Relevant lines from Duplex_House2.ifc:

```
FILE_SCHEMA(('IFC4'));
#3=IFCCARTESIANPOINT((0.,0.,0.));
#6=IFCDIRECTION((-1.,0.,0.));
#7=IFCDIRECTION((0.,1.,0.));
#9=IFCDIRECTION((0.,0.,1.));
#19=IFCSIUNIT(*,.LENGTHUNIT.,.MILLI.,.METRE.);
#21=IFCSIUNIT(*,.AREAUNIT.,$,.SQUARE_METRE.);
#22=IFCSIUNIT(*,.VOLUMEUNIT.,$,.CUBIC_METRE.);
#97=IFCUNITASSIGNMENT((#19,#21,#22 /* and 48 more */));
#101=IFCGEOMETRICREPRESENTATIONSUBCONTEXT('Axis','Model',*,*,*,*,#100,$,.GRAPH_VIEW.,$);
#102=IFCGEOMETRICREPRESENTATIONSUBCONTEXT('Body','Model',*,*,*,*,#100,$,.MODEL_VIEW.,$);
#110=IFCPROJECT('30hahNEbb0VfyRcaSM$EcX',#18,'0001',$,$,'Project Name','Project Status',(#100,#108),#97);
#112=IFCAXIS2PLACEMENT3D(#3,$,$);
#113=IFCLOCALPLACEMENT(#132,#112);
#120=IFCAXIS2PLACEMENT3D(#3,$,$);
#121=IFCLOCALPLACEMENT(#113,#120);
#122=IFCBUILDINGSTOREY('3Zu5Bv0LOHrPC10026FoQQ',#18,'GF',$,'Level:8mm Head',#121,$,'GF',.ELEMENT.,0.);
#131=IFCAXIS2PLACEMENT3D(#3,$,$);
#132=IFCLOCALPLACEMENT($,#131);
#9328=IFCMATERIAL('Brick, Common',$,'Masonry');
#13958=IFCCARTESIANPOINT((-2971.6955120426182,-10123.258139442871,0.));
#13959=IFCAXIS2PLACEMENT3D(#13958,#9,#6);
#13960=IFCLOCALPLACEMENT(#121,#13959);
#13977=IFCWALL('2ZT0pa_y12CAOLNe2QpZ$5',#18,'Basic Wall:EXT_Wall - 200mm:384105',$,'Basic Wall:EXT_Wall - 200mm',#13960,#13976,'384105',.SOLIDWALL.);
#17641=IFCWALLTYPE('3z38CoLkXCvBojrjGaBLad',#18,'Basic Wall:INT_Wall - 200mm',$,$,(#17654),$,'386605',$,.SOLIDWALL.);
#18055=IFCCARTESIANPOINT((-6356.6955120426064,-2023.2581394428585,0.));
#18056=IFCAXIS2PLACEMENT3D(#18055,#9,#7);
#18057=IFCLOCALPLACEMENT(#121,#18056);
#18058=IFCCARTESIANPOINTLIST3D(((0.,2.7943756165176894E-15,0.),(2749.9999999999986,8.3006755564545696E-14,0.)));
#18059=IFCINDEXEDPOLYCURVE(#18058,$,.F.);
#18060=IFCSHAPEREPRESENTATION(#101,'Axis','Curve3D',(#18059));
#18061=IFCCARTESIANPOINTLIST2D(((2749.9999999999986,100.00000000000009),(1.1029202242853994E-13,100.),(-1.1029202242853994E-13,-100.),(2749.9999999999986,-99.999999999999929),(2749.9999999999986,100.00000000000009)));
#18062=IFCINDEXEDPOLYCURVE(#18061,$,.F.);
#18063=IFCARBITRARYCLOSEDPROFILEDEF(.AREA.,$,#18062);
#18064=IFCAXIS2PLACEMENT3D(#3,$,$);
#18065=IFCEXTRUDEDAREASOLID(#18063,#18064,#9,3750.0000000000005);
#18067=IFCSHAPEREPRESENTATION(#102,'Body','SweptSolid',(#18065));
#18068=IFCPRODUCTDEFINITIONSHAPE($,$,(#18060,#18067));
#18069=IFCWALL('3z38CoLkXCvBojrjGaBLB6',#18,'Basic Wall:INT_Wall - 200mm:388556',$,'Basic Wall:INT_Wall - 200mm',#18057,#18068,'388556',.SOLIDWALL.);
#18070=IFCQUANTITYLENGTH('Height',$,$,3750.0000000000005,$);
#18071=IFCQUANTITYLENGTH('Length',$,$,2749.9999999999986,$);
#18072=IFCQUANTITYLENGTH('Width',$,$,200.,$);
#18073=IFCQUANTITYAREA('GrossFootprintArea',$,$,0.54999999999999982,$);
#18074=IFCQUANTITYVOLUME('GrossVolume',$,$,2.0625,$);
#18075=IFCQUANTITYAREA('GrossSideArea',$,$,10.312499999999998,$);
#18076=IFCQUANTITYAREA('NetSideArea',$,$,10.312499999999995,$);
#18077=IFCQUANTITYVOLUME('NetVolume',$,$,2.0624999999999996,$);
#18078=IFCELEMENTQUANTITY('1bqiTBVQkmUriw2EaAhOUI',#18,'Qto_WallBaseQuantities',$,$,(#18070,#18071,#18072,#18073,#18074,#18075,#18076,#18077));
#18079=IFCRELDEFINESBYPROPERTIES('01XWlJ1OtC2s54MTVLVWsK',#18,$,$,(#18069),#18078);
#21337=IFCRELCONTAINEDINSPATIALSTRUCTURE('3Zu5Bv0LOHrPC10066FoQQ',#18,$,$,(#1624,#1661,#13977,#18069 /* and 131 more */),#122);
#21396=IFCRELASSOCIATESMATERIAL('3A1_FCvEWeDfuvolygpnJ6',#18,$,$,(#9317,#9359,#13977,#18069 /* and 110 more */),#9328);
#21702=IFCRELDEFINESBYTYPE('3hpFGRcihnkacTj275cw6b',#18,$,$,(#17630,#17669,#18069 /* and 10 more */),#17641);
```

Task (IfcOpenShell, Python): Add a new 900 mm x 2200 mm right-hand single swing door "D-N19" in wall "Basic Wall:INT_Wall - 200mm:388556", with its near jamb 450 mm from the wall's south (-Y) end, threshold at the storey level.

```python
import numpy as np
import ifcopenshell
import ifcopenshell.api.feature
import ifcopenshell.api.geometry
import ifcopenshell.api.pset
import ifcopenshell.api.root
import ifcopenshell.api.spatial
import ifcopenshell.geom
import ifcopenshell.util.element
import ifcopenshell.util.placement
import ifcopenshell.util.representation
import ifcopenshell.util.shape
import ifcopenshell.util.unit

model = ifcopenshell.open("Duplex_House2.ifc")
unit_scale = ifcopenshell.util.unit.calculate_unit_scale(model)
area_scale = ifcopenshell.util.unit.calculate_unit_scale(model, "AREAUNIT")
volume_scale = ifcopenshell.util.unit.calculate_unit_scale(model, "VOLUMEUNIT")
settings = ifcopenshell.geom.settings()


def volume(element):
    """Net volume in cubic metres, openings subtracted."""
    shape = ifcopenshell.geom.create_shape(settings, element)
    return ifcopenshell.util.shape.get_volume(shape.geometry)


wall = model.by_guid("3z38CoLkXCvBojrjGaBLB6")
storey = ifcopenshell.util.element.get_container(wall, ifc_class="IfcBuildingStorey")
context = ifcopenshell.util.representation.get_context(model, "Model", "Body", "MODEL_VIEW")
before = volume(wall)

width, height, from_end, sill = 0.9, 2.2, 0.45, 0.0  # metres

# The wall runs along its own X axis, and the end named is its -X end.
wall_shape = ifcopenshell.geom.create_shape(settings, wall)
x, y, z = ifcopenshell.util.shape.get_vertices(wall_shape.geometry).T
start = x.min() + from_end
face, thickness = float(y.min()), float(y.max() - y.min())
wall_matrix = ifcopenshell.util.placement.get_local_placement(wall.ObjectPlacement)
level = ifcopenshell.util.placement.get_local_placement(storey.ObjectPlacement)[2, 3]


def in_wall(x, y):
    """Placement at x, y metres in the wall's axes, at sill height."""
    matrix = wall_matrix.copy()
    matrix[:, 3] = wall_matrix @ np.array([x / unit_scale, y / unit_scale, 0.0, 1.0])
    matrix[2, 3] = level + sill / unit_scale
    return matrix


# Opening: a box that overshoots both wall faces by 50 mm.
opening = ifcopenshell.api.root.create_entity(model, ifc_class="IfcOpeningElement", predefined_type="OPENING")
box = ifcopenshell.api.geometry.add_wall_representation(
    model, context=context, length=width, height=height, thickness=thickness + 0.1
)
ifcopenshell.api.geometry.assign_representation(model, product=opening, representation=box)
ifcopenshell.api.geometry.edit_object_placement(model, product=opening, matrix=in_wall(start, face - 0.05), is_si=False)
ifcopenshell.api.feature.add_feature(model, feature=opening, element=wall)

door = ifcopenshell.api.root.create_entity(model, ifc_class="IfcDoor", name="D-N19", predefined_type="DOOR")
door.OverallWidth, door.OverallHeight = width / unit_scale, height / unit_scale
door.OperationType = "SINGLE_SWING_RIGHT"
body = ifcopenshell.api.geometry.add_door_representation(
    model,
    context=context,
    overall_width=door.OverallWidth,
    overall_height=door.OverallHeight,
    operation_type="SINGLE_SWING_RIGHT",
    lining_properties={"LiningDepth": thickness / unit_scale, "ThresholdDepth": thickness / unit_scale},
)
ifcopenshell.api.geometry.assign_representation(model, product=door, representation=body)
ifcopenshell.api.spatial.assign_container(model, products=[door], relating_structure=storey)
ifcopenshell.api.feature.add_filling(model, opening=opening, element=door)

# The lining spans the wall, so the door starts at the wall face.
ifcopenshell.api.geometry.edit_object_placement(model, product=door, matrix=in_wall(start, face), is_si=False)

after = volume(wall)

# Update the wall's stored quantities.
qto = model.by_id(ifcopenshell.util.element.get_pset(wall, "Qto_WallBaseQuantities", should_inherit=False)["id"])
ifcopenshell.api.pset.edit_qto(model, qto=qto, properties={
    "NetSideArea": after / thickness / area_scale,
    "NetVolume": after / volume_scale,
})

print(f"wall volume {before:.3f} -> {after:.3f} m3")

model.write("Duplex_House2_updated.ifc")
```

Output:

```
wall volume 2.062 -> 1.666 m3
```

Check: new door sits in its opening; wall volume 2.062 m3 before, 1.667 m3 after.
